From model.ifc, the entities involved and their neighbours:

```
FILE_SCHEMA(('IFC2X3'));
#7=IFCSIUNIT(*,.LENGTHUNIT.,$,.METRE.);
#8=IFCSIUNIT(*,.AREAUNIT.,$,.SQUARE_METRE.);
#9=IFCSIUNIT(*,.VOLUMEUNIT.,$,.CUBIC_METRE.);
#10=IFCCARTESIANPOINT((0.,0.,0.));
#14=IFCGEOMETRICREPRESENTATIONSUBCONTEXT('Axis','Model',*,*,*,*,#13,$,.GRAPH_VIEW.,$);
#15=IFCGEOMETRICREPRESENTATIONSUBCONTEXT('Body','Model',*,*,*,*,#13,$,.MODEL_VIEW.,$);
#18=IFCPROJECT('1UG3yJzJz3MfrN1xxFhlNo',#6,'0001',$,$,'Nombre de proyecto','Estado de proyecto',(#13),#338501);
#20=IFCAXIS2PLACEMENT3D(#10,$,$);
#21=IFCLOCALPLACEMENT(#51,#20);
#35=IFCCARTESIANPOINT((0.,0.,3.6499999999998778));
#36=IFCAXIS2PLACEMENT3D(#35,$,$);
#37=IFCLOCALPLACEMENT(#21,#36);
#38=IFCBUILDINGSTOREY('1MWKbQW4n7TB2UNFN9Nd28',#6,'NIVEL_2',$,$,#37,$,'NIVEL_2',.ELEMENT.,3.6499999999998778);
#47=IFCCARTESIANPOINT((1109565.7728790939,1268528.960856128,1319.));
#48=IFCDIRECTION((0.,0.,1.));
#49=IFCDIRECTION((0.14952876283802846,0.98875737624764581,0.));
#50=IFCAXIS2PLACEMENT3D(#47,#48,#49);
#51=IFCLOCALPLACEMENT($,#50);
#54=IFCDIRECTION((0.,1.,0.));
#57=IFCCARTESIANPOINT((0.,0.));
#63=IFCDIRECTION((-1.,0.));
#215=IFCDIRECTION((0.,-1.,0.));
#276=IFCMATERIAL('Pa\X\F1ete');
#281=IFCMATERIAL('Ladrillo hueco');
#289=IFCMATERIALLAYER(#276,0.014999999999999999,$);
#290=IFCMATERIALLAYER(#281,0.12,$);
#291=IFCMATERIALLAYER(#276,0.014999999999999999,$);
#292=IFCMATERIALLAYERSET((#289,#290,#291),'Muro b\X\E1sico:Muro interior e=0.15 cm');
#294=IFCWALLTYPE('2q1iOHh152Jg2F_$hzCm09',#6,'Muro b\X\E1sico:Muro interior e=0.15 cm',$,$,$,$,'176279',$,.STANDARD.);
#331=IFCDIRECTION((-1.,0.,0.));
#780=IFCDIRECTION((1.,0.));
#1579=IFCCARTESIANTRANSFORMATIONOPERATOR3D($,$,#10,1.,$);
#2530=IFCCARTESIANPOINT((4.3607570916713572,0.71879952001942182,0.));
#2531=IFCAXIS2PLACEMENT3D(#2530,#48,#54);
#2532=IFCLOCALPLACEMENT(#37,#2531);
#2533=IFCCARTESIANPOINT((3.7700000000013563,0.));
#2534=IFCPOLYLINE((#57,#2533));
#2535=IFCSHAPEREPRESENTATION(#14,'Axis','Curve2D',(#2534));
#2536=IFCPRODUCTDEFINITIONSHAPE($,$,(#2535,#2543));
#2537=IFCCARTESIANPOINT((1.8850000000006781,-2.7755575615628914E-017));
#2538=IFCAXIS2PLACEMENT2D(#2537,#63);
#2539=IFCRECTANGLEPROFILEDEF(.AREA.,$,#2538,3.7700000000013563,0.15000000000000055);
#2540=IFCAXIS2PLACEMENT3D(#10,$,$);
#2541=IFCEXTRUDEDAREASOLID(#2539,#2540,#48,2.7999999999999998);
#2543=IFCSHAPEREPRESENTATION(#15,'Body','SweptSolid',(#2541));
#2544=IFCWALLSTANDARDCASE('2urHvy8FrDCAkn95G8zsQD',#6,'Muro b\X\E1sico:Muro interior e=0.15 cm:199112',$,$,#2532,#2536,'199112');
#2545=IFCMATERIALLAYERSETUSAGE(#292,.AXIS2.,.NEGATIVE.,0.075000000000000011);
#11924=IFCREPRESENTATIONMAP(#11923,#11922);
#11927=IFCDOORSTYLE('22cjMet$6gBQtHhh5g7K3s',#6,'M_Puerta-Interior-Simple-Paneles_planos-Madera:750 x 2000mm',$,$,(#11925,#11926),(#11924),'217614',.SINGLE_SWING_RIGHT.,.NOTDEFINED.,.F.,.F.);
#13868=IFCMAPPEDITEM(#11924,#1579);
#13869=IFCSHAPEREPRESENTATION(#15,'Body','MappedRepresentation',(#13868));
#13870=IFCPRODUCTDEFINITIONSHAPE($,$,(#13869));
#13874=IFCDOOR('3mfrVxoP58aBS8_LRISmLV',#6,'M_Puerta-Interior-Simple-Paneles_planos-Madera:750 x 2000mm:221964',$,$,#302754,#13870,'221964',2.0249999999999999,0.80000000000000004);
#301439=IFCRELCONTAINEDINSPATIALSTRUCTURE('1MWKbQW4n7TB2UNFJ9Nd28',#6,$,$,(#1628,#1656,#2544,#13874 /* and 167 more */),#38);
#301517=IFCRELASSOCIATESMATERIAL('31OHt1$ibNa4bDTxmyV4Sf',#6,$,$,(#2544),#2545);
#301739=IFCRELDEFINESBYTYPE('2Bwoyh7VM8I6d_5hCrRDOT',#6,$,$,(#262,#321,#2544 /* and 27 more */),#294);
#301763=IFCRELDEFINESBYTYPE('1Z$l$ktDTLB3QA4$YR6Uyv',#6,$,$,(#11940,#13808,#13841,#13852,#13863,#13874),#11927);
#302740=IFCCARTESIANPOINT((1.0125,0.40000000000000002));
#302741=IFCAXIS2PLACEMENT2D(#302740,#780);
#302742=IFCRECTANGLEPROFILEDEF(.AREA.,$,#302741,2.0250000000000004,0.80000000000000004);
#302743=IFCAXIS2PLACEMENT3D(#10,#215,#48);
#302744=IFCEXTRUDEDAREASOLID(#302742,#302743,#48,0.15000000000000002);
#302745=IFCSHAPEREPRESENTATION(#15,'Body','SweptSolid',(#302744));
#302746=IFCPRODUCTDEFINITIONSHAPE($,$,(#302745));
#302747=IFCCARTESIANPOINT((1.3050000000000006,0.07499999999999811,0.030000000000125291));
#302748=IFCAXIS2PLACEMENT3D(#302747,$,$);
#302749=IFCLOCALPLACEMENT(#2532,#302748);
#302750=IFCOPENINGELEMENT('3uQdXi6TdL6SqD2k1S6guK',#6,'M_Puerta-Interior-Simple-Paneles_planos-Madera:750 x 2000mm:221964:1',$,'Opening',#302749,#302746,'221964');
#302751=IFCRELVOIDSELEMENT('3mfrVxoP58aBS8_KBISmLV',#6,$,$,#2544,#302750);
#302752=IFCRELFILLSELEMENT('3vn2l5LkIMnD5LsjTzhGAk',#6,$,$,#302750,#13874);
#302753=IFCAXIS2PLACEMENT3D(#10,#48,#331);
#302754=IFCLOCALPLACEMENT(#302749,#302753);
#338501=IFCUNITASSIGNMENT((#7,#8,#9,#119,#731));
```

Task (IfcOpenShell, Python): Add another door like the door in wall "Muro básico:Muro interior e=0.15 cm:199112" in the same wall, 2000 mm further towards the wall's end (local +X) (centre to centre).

```python
import ifcopenshell
import ifcopenshell.api.feature
import ifcopenshell.api.geometry
import ifcopenshell.api.root
import ifcopenshell.geom
import ifcopenshell.util.element
import ifcopenshell.util.placement
import ifcopenshell.util.shape
import ifcopenshell.util.unit

model = ifcopenshell.open("model.ifc")
unit_scale = ifcopenshell.util.unit.calculate_unit_scale(model)
settings = ifcopenshell.geom.settings()


def volume(element):
    """Net volume in cubic metres, openings subtracted."""
    shape = ifcopenshell.geom.create_shape(settings, element)
    return ifcopenshell.util.shape.get_volume(shape.geometry)


def reuse_history(source, copy):
    """copy_class also copies each property set's owner history, people and application; keep the originals."""
    for rel in copy.IsDefinedBy:
        if rel.is_a("IfcRelDefinesByProperties") and (history := rel.RelatingPropertyDefinition.OwnerHistory):
            rel.RelatingPropertyDefinition.OwnerHistory = source.OwnerHistory
            ifcopenshell.util.element.remove_deep2(model, history)


door = model.by_guid("3mfrVxoP58aBS8_LRISmLV")
opening = door.FillsVoids[0].RelatingOpeningElement
wall = opening.VoidsElements[0].RelatingBuildingElement
before = volume(wall)
shift = ifcopenshell.util.placement.get_local_placement(wall.ObjectPlacement)[:3, 0] * 2 / unit_scale

# copy_class copies the void relationship, type, container and properties, but no geometry.
new_opening = ifcopenshell.api.root.copy_class(model, product=opening)
new_opening.Representation = ifcopenshell.util.element.copy_deep(
    model, opening.Representation, exclude=["IfcGeometricRepresentationContext", "IfcRepresentationMap"]
)
new_opening.Name = "M_Puerta-Interior-Simple-Paneles_planos-Madera:750 x 2000mm"
new_opening.Tag = None
new_door = ifcopenshell.api.root.copy_class(model, product=door)
new_door.Representation = ifcopenshell.util.element.copy_deep(
    model, door.Representation, exclude=["IfcGeometricRepresentationContext", "IfcRepresentationMap"]
)
new_door.Name = "M_Puerta-Interior-Simple-Paneles_planos-Madera:750 x 2000mm"
new_door.Tag = None
reuse_history(door, new_door)
fills = ifcopenshell.api.feature.add_filling(model, opening=new_opening, element=new_door)
fills.OwnerHistory = new_door.OwnerHistory  # required in IFC2X3

for old, new in ((opening, new_opening), (door, new_door)):
    matrix = ifcopenshell.util.placement.get_local_placement(old.ObjectPlacement)
    matrix[:3, 3] += shift
    ifcopenshell.api.geometry.edit_object_placement(model, product=new, matrix=matrix, is_si=False)

after = volume(wall)

print(f"wall volume {before:.3f} -> {after:.3f} m3")

model.write("model_v2.ifc")
```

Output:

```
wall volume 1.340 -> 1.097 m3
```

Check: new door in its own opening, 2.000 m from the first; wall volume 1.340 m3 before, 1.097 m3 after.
